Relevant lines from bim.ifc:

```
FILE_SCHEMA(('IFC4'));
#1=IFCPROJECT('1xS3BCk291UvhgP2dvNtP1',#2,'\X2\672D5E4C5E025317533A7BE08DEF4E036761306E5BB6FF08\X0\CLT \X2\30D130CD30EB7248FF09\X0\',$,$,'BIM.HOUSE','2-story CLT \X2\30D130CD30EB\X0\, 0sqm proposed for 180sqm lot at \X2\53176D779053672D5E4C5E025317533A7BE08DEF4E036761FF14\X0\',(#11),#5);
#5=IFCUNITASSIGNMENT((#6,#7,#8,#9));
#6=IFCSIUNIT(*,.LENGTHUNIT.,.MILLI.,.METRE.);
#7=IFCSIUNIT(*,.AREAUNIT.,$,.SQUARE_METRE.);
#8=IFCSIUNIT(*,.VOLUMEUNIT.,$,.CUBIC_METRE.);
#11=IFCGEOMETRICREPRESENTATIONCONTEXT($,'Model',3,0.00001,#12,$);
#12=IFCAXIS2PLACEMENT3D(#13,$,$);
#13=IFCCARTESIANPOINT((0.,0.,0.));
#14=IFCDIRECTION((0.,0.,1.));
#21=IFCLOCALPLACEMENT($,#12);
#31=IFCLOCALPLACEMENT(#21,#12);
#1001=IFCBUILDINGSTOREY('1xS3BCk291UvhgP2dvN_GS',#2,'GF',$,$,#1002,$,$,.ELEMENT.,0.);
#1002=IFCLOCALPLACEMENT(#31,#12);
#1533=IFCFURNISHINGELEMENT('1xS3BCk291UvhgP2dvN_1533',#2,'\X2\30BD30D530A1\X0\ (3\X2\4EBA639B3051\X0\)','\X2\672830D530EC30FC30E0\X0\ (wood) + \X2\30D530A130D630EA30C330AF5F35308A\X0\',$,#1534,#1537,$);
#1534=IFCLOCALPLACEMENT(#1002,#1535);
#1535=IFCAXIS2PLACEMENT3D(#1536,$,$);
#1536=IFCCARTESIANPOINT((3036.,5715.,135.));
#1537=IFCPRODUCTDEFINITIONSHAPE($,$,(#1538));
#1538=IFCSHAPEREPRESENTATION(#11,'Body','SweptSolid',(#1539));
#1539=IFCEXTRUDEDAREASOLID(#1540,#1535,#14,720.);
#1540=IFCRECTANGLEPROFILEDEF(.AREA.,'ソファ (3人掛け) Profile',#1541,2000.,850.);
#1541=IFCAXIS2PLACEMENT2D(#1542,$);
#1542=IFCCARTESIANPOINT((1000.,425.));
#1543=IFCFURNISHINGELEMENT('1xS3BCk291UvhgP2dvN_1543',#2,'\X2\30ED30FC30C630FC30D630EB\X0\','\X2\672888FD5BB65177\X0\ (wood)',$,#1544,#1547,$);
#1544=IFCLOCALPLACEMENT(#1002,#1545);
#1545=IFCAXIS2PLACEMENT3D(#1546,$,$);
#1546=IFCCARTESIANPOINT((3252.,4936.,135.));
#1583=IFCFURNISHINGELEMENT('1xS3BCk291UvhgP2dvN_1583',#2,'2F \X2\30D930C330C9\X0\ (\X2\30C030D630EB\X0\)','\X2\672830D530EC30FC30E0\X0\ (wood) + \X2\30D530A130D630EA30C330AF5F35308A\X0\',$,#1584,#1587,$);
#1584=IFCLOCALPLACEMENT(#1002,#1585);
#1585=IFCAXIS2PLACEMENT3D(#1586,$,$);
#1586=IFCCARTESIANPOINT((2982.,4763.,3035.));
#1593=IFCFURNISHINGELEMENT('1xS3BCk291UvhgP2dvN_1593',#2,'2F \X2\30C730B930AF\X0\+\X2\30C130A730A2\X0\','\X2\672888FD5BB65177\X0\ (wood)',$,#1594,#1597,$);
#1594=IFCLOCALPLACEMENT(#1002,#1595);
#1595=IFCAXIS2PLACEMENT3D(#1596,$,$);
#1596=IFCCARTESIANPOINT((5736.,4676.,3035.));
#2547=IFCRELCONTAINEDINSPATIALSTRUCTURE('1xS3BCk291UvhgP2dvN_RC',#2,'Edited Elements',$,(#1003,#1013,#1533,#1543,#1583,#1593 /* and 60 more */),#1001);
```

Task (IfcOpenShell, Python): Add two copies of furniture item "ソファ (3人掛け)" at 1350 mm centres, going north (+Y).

```python
import numpy as np
import ifcopenshell
import ifcopenshell.api.geometry
import ifcopenshell.api.root
import ifcopenshell.util.element
import ifcopenshell.util.placement
import ifcopenshell.util.unit

model = ifcopenshell.open("bim.ifc")
unit_scale = ifcopenshell.util.unit.calculate_unit_scale(model)


def reuse_history(source, copy):
    """copy_class also copies each property set's owner history, people and application; keep the originals."""
    for rel in copy.IsDefinedBy:
        if rel.is_a("IfcRelDefinesByProperties") and (history := rel.RelatingPropertyDefinition.OwnerHistory):
            rel.RelatingPropertyDefinition.OwnerHistory = source.OwnerHistory
            ifcopenshell.util.element.remove_deep2(model, history)


source = model.by_guid("1xS3BCk291UvhgP2dvN_1533")
base = ifcopenshell.util.placement.get_local_placement(source.ObjectPlacement)
step = np.array([0.0, 1.0, 0.0]) * 1.35 / unit_scale

for i in range(1, 3):
    copy = ifcopenshell.api.root.copy_class(model, product=source)
    copy.Representation = ifcopenshell.util.element.copy_deep(
        model, source.Representation, exclude=["IfcGeometricRepresentationContext", "IfcRepresentationMap"]
    )
    reuse_history(source, copy)
    matrix = base.copy()
    matrix[:3, 3] += i * step
    print("added at", matrix[:3, 3].round(3) + 0.0)
    ifcopenshell.api.geometry.edit_object_placement(model, product=copy, matrix=matrix, is_si=False)

model.write("bim_rev.ifc")
```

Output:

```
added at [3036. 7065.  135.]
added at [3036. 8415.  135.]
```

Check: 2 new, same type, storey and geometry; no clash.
